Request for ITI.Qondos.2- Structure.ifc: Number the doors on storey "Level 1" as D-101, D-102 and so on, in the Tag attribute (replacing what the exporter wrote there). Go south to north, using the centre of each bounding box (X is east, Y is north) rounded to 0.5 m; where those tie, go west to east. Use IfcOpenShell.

First a look at what the model holds.

```python
import ifcopenshell
import ifcopenshell.util.element
import ifcopenshell.util.placement

model = ifcopenshell.open("ITI.Qondos.2- Structure.ifc")
print(model.schema)
storey = next(s for s in model.by_type("IfcBuildingStorey") if s.Name == "Level 1")
doors = [e for e in ifcopenshell.util.element.get_decomposition(storey) if e.is_a("IfcDoor")]
for e in sorted(doors, key=lambda e: e.id()):
    origin = ifcopenshell.util.placement.get_local_placement(e.ObjectPlacement)[:3, 3]
    print(e.id(), e.Tag, e.Name, origin.round(2) + 0.0, sep=" | ")
```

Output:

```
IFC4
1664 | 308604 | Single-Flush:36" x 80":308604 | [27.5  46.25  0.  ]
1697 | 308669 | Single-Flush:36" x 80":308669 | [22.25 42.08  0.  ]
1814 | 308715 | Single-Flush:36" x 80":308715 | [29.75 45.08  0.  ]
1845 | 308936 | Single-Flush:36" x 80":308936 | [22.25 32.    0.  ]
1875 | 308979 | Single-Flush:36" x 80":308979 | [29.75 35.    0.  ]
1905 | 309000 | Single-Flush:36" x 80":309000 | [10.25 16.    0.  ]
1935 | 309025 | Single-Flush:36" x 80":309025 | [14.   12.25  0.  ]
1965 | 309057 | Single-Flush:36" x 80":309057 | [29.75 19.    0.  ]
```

```python
import ifcopenshell
import ifcopenshell.geom
import ifcopenshell.util.element
import ifcopenshell.util.shape

model = ifcopenshell.open("ITI.Qondos.2- Structure.ifc")
settings = ifcopenshell.geom.settings()
settings.set("use-world-coords", True)


def centre(element):
    shape = ifcopenshell.geom.create_shape(settings, element)
    return ifcopenshell.util.shape.get_bbox_centroid(shape.geometry)


storey = next(s for s in model.by_type("IfcBuildingStorey") if s.Name == "Level 1")
doors = [e for e in ifcopenshell.util.element.get_decomposition(storey) if e.is_a("IfcDoor")]

# Insertion points can sit at a corner or the storey origin, so sort by the geometry (in metres).
centres = {e: centre(e) for e in doors}
doors.sort(key=lambda e: (round(centres[e][1] / 0.5), centres[e][0]))

for i, e in enumerate(doors, start=1):
    number = f"D-1{i:02d}"
    e.Tag = number
    print(e.id(), number)

model.write("ITI.Qondos.2- Structure_updated.ifc")
```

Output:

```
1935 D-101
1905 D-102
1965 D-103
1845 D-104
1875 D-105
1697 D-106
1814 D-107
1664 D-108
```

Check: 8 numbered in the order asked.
